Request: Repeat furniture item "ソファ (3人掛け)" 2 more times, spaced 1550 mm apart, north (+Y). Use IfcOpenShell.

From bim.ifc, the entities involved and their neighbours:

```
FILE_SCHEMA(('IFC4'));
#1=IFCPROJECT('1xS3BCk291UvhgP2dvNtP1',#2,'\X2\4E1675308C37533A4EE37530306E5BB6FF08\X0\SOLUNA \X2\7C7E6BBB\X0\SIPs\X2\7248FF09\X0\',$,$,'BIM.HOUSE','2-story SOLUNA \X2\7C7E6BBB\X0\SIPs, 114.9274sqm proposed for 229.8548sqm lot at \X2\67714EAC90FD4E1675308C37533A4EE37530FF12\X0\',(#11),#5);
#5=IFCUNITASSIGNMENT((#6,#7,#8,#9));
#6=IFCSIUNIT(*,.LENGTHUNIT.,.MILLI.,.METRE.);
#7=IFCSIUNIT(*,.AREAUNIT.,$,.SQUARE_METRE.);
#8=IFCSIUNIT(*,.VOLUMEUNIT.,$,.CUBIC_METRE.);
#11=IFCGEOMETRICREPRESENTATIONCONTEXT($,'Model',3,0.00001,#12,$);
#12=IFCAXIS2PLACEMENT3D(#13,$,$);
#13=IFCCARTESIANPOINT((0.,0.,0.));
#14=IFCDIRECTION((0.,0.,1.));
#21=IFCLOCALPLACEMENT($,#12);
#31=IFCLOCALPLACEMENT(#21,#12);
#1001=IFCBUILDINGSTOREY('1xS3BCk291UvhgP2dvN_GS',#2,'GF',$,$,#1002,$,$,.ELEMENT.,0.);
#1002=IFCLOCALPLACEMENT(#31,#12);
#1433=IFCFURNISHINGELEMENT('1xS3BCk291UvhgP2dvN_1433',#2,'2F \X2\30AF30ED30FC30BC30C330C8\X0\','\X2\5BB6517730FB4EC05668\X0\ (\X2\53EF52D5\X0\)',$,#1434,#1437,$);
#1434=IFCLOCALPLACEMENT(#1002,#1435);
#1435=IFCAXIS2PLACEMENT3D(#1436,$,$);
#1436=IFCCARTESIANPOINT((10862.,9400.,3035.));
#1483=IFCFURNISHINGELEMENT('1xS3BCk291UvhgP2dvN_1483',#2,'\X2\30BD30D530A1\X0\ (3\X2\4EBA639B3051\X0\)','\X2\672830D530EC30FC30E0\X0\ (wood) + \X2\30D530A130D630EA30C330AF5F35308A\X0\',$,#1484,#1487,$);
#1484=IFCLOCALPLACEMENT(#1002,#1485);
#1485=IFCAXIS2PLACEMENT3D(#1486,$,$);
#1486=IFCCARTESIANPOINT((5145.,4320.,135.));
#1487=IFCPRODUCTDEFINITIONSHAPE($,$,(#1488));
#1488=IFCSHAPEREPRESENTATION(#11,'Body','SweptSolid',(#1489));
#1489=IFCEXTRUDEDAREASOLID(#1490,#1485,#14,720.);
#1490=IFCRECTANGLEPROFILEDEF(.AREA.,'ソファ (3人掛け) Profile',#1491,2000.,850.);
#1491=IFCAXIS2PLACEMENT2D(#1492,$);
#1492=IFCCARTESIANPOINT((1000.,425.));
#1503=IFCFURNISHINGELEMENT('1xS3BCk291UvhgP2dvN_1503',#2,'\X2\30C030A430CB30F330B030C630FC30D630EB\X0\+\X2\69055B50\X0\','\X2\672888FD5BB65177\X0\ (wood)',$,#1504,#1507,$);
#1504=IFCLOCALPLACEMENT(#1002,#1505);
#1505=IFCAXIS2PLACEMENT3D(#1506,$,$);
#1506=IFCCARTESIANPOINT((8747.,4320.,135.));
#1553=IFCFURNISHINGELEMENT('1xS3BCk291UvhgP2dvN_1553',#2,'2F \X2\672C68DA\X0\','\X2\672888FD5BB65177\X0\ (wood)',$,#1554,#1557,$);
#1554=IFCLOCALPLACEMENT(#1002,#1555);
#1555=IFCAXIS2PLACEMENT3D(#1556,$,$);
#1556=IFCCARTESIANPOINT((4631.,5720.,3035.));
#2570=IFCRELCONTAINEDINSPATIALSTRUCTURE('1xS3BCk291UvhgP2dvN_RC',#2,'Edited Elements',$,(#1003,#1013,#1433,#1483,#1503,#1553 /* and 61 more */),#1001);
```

```python
import numpy as np
import ifcopenshell
import ifcopenshell.api.geometry
import ifcopenshell.api.root
import ifcopenshell.util.element
import ifcopenshell.util.placement
import ifcopenshell.util.unit

model = ifcopenshell.open("bim.ifc")
unit_scale = ifcopenshell.util.unit.calculate_unit_scale(model)


def reuse_history(source, copy):
    """copy_class also copies each property set's owner history, people and application; keep the originals."""
    for rel in copy.IsDefinedBy:
        if rel.is_a("IfcRelDefinesByProperties") and (history := rel.RelatingPropertyDefinition.OwnerHistory):
            rel.RelatingPropertyDefinition.OwnerHistory = source.OwnerHistory
            ifcopenshell.util.element.remove_deep2(model, history)


source = model.by_id(1483)
base = ifcopenshell.util.placement.get_local_placement(source.ObjectPlacement)
step = np.array([0.0, 1.0, 0.0]) * 1.55 / unit_scale

for i in range(1, 3):
    copy = ifcopenshell.api.root.copy_class(model, product=source)
    copy.Representation = ifcopenshell.util.element.copy_deep(
        model, source.Representation, exclude=["IfcGeometricRepresentationContext", "IfcRepresentationMap"]
    )
    reuse_history(source, copy)
    matrix = base.copy()
    matrix[:3, 3] += i * step
    print("added at", matrix[:3, 3].round(3) + 0.0)
    ifcopenshell.api.geometry.edit_object_placement(model, product=copy, matrix=matrix, is_si=False)

model.write("bim_updated.ifc")
```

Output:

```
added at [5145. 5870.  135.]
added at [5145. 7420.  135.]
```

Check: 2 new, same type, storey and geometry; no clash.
